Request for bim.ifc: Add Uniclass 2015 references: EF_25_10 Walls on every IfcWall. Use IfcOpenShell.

First a look at what the model holds.

```python
import ifcopenshell

model = ifcopenshell.open("bim.ifc")
print(model.schema)
print("classifications:", [c.Name for c in model.by_type("IfcClassification")])
for ifc_class in ("IfcDoor", "IfcRoof", "IfcStair", "IfcWall", "IfcWindow"):
    print(ifc_class, len(model.by_type(ifc_class)))
```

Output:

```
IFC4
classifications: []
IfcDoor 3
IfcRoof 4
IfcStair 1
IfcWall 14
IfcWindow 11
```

```python
import ifcopenshell
import ifcopenshell.api.classification

model = ifcopenshell.open("bim.ifc")

system = ifcopenshell.api.classification.add_classification(model, classification="Uniclass 2015")

codes = {
    "IfcWall": ("EF_25_10", "Walls"),
}
for ifc_class, (code, name) in codes.items():
    products = model.by_type(ifc_class)
    ifcopenshell.api.classification.add_reference(
        model, products=products, classification=system, identification=code, name=name
    )
    print(code, len(products))

model.write("bim_rev.ifc")
```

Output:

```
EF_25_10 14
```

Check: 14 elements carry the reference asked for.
